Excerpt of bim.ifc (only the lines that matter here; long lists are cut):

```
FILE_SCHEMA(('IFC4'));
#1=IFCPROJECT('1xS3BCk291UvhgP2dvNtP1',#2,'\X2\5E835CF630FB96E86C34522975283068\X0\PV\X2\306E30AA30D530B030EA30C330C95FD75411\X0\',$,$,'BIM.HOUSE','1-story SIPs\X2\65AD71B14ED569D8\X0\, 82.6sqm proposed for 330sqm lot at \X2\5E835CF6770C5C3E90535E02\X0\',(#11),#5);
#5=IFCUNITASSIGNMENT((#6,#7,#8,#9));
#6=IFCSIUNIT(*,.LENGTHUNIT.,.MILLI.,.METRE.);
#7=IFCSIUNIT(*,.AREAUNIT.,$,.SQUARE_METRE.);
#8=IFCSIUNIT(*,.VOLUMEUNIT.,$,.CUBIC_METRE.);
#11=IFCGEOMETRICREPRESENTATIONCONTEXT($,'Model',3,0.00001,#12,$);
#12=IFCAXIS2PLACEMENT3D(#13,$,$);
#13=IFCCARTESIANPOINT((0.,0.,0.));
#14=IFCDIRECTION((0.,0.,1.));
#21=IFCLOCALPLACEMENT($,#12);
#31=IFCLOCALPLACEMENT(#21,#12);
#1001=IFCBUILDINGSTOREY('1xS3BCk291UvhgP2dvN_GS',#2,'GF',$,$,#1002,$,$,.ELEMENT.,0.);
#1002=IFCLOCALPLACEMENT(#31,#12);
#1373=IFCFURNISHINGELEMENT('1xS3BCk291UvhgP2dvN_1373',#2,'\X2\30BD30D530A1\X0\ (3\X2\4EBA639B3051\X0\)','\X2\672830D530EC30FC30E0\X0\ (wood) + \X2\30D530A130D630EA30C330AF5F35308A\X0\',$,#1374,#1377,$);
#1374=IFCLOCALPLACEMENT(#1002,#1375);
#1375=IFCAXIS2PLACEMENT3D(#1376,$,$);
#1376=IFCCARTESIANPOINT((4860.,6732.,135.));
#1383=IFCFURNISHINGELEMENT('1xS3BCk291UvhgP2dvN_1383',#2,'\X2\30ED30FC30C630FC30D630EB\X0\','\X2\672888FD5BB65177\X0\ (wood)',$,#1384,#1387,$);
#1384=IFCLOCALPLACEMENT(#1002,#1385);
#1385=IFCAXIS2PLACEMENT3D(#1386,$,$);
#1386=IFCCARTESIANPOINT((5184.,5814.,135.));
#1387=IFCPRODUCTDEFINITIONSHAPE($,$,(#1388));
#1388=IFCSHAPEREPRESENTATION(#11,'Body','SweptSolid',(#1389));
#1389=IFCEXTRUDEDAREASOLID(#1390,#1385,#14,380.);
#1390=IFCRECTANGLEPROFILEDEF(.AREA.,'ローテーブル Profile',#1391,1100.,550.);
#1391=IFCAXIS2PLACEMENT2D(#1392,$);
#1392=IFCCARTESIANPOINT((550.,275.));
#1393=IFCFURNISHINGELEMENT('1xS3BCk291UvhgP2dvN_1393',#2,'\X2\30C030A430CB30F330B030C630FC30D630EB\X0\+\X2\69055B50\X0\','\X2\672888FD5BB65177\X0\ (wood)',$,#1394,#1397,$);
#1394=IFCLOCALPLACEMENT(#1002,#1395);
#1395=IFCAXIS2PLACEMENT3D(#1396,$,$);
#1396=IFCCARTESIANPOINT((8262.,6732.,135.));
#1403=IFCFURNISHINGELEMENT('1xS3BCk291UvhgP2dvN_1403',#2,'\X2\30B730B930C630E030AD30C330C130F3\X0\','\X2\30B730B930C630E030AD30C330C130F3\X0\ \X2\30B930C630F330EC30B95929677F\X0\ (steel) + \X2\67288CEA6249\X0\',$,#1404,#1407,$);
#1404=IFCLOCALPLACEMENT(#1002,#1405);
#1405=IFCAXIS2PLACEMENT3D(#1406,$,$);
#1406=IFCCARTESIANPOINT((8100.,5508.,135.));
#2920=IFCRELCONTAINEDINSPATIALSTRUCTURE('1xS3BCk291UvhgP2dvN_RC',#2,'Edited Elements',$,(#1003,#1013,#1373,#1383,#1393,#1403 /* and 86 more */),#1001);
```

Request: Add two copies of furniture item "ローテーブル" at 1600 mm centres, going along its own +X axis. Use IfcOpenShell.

```python
import ifcopenshell
import ifcopenshell.api.geometry
import ifcopenshell.api.root
import ifcopenshell.util.element
import ifcopenshell.util.placement

model = ifcopenshell.open("bim.ifc")


def reuse_history(source, copy):
    """copy_class also copies each property set's owner history, people and application; keep the originals."""
    for rel in copy.IsDefinedBy:
        if rel.is_a("IfcRelDefinesByProperties") and (history := rel.RelatingPropertyDefinition.OwnerHistory):
            rel.RelatingPropertyDefinition.OwnerHistory = source.OwnerHistory
            ifcopenshell.util.element.remove_deep2(model, history)


source = model.by_guid("1xS3BCk291UvhgP2dvN_1383")
base = ifcopenshell.util.placement.get_local_placement(source.ObjectPlacement)
step = base[:3, 0] * 1600.0

for i in range(1, 3):
    copy = ifcopenshell.api.root.copy_class(model, product=source)
    copy.Representation = ifcopenshell.util.element.copy_deep(
        model, source.Representation, exclude=["IfcGeometricRepresentationContext", "IfcRepresentationMap"]
    )
    reuse_history(source, copy)
    matrix = base.copy()
    matrix[:3, 3] += i * step
    print("added at", matrix[:3, 3].round(3) + 0.0)
    ifcopenshell.api.geometry.edit_object_placement(model, product=copy, matrix=matrix, is_si=False)

model.write("bim_edited.ifc")
```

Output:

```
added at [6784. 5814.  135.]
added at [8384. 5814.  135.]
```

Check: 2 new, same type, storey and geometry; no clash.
